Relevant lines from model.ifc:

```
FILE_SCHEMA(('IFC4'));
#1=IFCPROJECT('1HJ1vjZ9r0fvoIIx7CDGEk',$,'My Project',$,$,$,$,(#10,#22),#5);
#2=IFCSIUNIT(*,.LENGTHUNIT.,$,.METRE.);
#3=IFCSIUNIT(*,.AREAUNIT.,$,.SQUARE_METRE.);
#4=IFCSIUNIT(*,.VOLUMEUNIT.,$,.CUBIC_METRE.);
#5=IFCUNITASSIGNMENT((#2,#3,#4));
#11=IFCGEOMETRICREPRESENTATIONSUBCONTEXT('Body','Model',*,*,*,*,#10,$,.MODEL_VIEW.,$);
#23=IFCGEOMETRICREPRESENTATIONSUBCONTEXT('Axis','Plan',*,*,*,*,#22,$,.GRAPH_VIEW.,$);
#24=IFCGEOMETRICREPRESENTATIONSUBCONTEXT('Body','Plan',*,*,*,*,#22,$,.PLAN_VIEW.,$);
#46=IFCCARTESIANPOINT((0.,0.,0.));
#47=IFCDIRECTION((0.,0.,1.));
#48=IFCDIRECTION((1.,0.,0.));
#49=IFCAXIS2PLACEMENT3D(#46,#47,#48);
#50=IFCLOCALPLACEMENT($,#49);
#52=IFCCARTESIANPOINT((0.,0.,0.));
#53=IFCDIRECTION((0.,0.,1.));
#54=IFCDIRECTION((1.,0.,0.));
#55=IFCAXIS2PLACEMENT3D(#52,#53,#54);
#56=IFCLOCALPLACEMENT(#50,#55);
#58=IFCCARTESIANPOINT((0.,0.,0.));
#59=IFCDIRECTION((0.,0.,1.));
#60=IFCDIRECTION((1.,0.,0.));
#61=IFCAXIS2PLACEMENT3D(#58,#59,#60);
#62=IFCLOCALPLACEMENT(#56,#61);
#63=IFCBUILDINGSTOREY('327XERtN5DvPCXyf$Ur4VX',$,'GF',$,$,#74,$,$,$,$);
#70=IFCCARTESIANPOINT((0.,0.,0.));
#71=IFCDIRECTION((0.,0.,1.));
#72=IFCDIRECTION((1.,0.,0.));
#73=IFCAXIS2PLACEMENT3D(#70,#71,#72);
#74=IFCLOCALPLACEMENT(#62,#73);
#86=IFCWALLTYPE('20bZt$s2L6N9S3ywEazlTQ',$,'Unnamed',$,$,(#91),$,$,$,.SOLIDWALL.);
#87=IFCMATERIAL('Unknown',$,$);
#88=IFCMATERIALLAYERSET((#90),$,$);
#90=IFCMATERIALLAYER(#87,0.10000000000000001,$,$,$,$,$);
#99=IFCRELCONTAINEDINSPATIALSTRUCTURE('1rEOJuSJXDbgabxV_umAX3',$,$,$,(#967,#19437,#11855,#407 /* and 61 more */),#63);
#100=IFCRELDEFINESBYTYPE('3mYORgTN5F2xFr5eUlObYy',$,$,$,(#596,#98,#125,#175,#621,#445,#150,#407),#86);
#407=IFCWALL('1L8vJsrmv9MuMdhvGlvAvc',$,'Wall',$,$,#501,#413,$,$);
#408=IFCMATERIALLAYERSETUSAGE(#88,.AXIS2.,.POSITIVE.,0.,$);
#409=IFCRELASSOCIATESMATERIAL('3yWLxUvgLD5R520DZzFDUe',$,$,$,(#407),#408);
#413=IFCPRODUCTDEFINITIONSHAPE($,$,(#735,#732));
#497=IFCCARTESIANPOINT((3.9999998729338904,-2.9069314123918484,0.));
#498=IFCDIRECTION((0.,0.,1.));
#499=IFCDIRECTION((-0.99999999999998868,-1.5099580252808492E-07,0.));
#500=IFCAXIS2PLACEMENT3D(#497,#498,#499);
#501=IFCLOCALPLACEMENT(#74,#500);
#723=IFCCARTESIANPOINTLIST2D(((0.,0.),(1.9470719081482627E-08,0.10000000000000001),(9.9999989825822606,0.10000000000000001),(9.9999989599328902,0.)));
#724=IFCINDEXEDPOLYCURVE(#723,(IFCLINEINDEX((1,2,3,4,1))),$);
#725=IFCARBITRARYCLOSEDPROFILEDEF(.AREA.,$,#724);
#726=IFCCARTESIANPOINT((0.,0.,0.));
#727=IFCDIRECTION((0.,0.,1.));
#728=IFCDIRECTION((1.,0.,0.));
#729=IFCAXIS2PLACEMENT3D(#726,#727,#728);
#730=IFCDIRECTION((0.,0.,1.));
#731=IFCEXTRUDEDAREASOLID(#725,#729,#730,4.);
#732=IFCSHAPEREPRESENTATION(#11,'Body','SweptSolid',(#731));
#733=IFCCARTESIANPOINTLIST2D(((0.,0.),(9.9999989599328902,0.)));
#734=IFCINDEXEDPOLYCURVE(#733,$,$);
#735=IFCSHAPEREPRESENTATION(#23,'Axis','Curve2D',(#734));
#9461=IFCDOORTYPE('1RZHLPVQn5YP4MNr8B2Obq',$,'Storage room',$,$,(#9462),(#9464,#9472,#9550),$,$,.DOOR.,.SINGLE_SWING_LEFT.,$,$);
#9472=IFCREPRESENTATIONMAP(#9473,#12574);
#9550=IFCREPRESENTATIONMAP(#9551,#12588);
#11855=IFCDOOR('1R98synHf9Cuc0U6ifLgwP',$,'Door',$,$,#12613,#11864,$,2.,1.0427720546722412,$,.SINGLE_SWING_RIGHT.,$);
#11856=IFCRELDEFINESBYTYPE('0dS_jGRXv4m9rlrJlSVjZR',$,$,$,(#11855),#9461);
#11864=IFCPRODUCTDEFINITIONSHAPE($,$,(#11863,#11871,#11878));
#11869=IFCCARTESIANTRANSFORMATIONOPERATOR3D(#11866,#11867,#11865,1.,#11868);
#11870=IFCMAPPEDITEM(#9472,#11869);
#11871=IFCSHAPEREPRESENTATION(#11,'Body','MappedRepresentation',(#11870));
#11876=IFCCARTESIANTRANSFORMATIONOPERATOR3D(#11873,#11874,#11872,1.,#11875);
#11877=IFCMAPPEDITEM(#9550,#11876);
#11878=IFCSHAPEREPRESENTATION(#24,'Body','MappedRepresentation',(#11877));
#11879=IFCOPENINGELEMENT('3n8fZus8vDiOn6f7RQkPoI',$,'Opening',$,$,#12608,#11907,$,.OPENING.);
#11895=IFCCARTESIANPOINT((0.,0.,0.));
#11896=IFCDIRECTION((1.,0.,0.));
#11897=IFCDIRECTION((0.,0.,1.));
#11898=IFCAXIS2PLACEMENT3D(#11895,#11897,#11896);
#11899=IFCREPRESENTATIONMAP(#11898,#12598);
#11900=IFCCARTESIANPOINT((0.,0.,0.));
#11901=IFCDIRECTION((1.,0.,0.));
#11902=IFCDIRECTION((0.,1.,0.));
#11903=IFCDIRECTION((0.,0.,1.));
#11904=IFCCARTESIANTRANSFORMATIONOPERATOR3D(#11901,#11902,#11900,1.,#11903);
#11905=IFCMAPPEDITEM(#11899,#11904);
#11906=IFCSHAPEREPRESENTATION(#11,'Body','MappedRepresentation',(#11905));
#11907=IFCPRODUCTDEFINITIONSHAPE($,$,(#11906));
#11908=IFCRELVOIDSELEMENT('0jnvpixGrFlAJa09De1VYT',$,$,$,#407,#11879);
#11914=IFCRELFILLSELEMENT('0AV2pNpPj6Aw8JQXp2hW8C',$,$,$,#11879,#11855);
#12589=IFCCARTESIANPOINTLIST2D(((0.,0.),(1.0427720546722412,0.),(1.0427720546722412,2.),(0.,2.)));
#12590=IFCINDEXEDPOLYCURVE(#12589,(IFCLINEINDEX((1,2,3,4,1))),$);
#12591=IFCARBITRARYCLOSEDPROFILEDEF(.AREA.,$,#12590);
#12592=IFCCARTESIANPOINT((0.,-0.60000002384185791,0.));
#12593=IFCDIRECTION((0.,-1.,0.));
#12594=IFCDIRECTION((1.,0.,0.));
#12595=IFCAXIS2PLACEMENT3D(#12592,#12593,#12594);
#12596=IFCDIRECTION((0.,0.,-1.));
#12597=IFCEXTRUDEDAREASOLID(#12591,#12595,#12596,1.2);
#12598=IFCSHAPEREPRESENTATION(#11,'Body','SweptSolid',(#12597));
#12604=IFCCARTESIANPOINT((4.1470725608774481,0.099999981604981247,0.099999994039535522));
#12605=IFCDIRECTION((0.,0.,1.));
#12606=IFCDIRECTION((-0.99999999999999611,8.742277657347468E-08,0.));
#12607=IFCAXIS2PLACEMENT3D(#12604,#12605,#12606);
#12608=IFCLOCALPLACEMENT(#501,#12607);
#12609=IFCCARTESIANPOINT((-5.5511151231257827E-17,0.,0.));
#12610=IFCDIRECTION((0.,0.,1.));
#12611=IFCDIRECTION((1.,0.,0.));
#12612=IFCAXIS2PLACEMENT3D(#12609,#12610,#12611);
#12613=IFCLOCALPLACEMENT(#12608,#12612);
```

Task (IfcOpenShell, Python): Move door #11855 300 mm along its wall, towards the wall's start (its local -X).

```python
import ifcopenshell
import ifcopenshell.api.geometry
import ifcopenshell.util.placement

model = ifcopenshell.open("model.ifc")

door = model.by_id(11855)
opening = door.FillsVoids[0].RelatingOpeningElement
wall = opening.VoidsElements[0].RelatingBuildingElement

wall_matrix = ifcopenshell.util.placement.get_local_placement(wall.ObjectPlacement)
shift = wall_matrix[:3, 0] * -0.3
before = ifcopenshell.util.placement.get_local_placement(door.ObjectPlacement)[:3, 3].copy()

# The door is placed relative to its opening, so it follows when the opening moves.
matrix = ifcopenshell.util.placement.get_local_placement(opening.ObjectPlacement)
matrix[:3, 3] += shift
ifcopenshell.api.geometry.edit_object_placement(
    model, product=opening, matrix=matrix, is_si=False, should_transform_children=True
)

after = ifcopenshell.util.placement.get_local_placement(door.ObjectPlacement)[:3, 3]
print("door moved by", (after - before).round(3) + 0.0)

model.write("model_edited.ifc")
```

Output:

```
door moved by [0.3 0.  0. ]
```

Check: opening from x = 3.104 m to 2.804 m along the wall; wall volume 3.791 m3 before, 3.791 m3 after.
